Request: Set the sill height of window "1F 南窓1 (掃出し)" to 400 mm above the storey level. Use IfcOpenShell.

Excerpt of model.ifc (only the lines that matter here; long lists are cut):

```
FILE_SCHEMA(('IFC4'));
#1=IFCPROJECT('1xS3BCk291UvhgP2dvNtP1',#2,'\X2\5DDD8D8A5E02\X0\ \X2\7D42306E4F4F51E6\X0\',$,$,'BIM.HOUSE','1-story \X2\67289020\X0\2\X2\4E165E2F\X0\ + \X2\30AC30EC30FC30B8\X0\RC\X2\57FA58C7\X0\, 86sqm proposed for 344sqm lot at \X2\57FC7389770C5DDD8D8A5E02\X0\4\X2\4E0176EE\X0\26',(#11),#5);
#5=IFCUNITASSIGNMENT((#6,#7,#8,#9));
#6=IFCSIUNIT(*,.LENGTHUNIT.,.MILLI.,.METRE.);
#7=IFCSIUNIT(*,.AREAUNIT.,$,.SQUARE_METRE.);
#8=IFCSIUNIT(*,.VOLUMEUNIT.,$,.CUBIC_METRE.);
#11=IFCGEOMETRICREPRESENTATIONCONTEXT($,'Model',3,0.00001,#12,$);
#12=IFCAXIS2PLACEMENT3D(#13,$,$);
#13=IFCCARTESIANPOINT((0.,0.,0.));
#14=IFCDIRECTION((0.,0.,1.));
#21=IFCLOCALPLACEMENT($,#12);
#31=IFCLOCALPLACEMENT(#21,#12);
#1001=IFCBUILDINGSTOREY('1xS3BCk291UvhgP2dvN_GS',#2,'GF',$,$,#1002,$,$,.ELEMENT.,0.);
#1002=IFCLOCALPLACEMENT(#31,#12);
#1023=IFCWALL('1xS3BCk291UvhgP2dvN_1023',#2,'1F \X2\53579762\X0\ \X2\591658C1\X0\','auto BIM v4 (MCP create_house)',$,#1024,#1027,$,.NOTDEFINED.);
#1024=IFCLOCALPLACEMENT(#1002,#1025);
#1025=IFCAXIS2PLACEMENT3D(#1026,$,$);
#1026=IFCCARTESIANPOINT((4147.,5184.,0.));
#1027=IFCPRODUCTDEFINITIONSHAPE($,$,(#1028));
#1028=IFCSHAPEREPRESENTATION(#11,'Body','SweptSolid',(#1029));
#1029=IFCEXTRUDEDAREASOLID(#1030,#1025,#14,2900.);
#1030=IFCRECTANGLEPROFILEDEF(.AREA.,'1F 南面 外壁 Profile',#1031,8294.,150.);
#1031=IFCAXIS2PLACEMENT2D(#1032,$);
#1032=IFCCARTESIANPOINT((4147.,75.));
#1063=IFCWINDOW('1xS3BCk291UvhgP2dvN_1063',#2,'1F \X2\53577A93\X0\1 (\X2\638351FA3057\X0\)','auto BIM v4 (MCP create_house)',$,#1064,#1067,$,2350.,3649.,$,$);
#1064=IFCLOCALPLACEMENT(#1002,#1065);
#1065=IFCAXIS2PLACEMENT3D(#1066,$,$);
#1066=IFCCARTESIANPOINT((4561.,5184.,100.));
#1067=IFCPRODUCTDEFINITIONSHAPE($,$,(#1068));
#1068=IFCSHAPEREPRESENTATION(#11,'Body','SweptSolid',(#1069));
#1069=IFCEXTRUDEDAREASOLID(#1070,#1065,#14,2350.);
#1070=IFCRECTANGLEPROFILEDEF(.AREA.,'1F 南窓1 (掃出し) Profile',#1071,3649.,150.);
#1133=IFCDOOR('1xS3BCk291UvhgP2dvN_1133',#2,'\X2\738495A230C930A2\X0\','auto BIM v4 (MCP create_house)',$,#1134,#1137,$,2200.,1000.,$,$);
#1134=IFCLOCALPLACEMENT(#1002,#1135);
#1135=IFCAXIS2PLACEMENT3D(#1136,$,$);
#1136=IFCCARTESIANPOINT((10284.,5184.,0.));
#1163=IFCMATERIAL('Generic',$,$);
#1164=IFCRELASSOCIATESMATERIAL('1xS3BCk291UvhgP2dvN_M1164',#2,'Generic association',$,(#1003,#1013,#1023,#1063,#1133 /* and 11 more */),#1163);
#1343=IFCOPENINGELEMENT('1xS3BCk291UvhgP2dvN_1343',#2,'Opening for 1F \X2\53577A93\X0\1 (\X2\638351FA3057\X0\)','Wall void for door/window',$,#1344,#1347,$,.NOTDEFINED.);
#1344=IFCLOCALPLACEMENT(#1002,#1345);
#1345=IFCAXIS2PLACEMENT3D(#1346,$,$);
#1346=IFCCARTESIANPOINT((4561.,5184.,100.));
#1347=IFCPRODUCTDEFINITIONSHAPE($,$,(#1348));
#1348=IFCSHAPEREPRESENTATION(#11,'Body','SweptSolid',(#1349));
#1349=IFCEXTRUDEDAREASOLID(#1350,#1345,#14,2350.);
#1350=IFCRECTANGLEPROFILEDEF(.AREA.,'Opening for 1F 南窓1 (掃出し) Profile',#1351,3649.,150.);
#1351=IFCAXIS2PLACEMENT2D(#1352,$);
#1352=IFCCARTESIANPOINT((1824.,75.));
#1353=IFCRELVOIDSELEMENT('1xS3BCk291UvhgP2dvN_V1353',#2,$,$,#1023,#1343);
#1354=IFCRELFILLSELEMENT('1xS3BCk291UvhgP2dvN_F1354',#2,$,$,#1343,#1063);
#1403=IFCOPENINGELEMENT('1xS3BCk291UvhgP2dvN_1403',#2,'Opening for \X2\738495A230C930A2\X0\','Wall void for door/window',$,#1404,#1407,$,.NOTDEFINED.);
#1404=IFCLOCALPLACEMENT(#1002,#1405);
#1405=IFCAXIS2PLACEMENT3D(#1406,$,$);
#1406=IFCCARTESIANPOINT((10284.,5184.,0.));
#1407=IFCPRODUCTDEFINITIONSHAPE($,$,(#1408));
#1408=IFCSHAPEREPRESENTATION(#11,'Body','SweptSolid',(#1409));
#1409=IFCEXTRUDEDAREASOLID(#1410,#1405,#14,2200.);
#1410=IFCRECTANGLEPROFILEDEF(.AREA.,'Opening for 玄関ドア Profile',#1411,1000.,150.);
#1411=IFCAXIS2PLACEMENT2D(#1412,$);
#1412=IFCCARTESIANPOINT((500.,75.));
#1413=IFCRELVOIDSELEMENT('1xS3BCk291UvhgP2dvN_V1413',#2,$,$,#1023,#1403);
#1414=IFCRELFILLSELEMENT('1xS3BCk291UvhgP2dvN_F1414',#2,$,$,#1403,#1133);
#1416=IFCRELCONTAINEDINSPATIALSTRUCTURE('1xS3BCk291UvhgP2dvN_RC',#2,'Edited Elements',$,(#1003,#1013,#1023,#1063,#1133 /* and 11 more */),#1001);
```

```python
import numpy as np
import ifcopenshell
import ifcopenshell.api.geometry
import ifcopenshell.geom
import ifcopenshell.util.element
import ifcopenshell.util.placement
import ifcopenshell.util.shape
import ifcopenshell.util.unit

model = ifcopenshell.open("model.ifc")
unit_scale = ifcopenshell.util.unit.calculate_unit_scale(model)

window = model.by_guid("1xS3BCk291UvhgP2dvN_1063")
opening = window.FillsVoids[0].RelatingOpeningElement
storey = ifcopenshell.util.element.get_container(window, ifc_class="IfcBuildingStorey")
level = ifcopenshell.util.placement.get_local_placement(storey.ObjectPlacement)[2, 3]

# The opening's origin need not be at the sill, so measure its lowest point.
shape = ifcopenshell.geom.create_shape(ifcopenshell.geom.settings(), opening)
bottom = ifcopenshell.util.shape.get_shape_bottom_elevation(shape, shape.geometry) / unit_scale
dz = level + 400.0 - bottom

shift = np.array([0.0, 0.0, dz])
# The window is not placed relative to its opening, so move both.
for product in (opening, window):
    matrix = ifcopenshell.util.placement.get_local_placement(product.ObjectPlacement)
    matrix[:3, 3] += shift
    ifcopenshell.api.geometry.edit_object_placement(model, product=product, matrix=matrix, is_si=False)

print(f"moved by {dz * unit_scale:+.3f} m")

model.write("model_v2.ifc")
```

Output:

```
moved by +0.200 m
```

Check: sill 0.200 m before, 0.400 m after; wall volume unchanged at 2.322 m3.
